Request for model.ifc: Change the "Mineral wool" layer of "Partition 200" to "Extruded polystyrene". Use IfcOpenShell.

First a look at what the model holds.

```python
import ifcopenshell
import ifcopenshell.util.element

model = ifcopenshell.open("model.ifc")
print(model.schema)
for layer_set in model.by_type("IfcMaterialLayerSet"):
    if layer_set.LayerSetName == "Partition 200":
        for layer in layer_set.MaterialLayers:
            print(layer.id(), layer.Material and layer.Material.Name, layer.LayerThickness, sep=" | ")
        print(len(ifcopenshell.util.element.get_elements_by_material(model, layer_set)), "elements and types use it")
print(sorted(m.Name for m in model.by_type("IfcMaterial") if m.Name)[:60])
```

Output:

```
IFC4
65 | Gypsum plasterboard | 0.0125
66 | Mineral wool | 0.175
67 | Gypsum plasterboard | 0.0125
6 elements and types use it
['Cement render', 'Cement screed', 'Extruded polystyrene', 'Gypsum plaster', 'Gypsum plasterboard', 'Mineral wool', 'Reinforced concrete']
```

```python
import ifcopenshell
import ifcopenshell.api.material

model = ifcopenshell.open("model.ifc")

layer_set = next(s for s in model.by_type("IfcMaterialLayerSet") if s.LayerSetName == "Partition 200")
layer = next(l for l in layer_set.MaterialLayers if l.Material and l.Material.Name == "Mineral wool")
material = next(m for m in model.by_type("IfcMaterial") if m.Name == "Extruded polystyrene")

# Point this one layer at the other material; renaming the old one would change it everywhere.
ifcopenshell.api.material.edit_layer(model, layer=layer, attributes={"Name": material.Name}, material=material)

print([l.Material.Name if l.Material else None for l in layer_set.MaterialLayers])

model.write("model_updated.ifc")
```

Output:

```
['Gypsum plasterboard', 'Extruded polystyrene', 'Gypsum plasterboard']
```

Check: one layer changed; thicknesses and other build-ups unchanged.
